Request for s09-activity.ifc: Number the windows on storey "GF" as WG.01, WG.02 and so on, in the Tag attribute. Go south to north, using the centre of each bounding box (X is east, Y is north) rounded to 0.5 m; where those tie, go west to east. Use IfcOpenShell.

First a look at what the model holds.

```python
import ifcopenshell
import ifcopenshell.util.element
import ifcopenshell.util.placement

model = ifcopenshell.open("s09-activity.ifc")
print(model.schema)
storey = next(s for s in model.by_type("IfcBuildingStorey") if s.Name == "GF")
windows = [e for e in ifcopenshell.util.element.get_decomposition(storey) if e.is_a("IfcWindow")]
for e in sorted(windows, key=lambda e: e.id()):
    origin = ifcopenshell.util.placement.get_local_placement(e.ObjectPlacement)[:3, 3]
    print(e.id(), e.Tag, e.Name, origin.round(2) + 0.0, sep=" | ")
```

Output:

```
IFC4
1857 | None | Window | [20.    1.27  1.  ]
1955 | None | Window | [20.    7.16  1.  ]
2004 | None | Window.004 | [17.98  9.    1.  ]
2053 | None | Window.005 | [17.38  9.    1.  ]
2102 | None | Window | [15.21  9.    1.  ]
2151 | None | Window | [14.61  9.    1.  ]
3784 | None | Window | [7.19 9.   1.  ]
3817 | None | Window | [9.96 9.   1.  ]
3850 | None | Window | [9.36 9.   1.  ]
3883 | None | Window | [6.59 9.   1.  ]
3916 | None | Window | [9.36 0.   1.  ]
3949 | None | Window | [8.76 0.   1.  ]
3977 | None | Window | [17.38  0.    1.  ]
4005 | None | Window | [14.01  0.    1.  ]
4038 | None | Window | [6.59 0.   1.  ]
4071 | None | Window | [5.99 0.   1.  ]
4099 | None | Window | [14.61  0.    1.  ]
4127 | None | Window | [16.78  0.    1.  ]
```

```python
import ifcopenshell
import ifcopenshell.geom
import ifcopenshell.util.element
import ifcopenshell.util.shape

model = ifcopenshell.open("s09-activity.ifc")
settings = ifcopenshell.geom.settings()
settings.set("use-world-coords", True)


def centre(element):
    shape = ifcopenshell.geom.create_shape(settings, element)
    return ifcopenshell.util.shape.get_bbox_centroid(shape.geometry)


storey = next(s for s in model.by_type("IfcBuildingStorey") if s.Name == "GF")
windows = [e for e in ifcopenshell.util.element.get_decomposition(storey) if e.is_a("IfcWindow")]

# Insertion points can sit at a corner or the storey origin, so sort by the geometry (in metres).
centres = {e: centre(e) for e in windows}
windows.sort(key=lambda e: (round(centres[e][1] / 0.5), centres[e][0]))

for i, e in enumerate(windows, start=1):
    number = f"WG.{i:02d}"
    e.Tag = number
    print(e.id(), number)

model.write("s09-activity_v2.ifc")
```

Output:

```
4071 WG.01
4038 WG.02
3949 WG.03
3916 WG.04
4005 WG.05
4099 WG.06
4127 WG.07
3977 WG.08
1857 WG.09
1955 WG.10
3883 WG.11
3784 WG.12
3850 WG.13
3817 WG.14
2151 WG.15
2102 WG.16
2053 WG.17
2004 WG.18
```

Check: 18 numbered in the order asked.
